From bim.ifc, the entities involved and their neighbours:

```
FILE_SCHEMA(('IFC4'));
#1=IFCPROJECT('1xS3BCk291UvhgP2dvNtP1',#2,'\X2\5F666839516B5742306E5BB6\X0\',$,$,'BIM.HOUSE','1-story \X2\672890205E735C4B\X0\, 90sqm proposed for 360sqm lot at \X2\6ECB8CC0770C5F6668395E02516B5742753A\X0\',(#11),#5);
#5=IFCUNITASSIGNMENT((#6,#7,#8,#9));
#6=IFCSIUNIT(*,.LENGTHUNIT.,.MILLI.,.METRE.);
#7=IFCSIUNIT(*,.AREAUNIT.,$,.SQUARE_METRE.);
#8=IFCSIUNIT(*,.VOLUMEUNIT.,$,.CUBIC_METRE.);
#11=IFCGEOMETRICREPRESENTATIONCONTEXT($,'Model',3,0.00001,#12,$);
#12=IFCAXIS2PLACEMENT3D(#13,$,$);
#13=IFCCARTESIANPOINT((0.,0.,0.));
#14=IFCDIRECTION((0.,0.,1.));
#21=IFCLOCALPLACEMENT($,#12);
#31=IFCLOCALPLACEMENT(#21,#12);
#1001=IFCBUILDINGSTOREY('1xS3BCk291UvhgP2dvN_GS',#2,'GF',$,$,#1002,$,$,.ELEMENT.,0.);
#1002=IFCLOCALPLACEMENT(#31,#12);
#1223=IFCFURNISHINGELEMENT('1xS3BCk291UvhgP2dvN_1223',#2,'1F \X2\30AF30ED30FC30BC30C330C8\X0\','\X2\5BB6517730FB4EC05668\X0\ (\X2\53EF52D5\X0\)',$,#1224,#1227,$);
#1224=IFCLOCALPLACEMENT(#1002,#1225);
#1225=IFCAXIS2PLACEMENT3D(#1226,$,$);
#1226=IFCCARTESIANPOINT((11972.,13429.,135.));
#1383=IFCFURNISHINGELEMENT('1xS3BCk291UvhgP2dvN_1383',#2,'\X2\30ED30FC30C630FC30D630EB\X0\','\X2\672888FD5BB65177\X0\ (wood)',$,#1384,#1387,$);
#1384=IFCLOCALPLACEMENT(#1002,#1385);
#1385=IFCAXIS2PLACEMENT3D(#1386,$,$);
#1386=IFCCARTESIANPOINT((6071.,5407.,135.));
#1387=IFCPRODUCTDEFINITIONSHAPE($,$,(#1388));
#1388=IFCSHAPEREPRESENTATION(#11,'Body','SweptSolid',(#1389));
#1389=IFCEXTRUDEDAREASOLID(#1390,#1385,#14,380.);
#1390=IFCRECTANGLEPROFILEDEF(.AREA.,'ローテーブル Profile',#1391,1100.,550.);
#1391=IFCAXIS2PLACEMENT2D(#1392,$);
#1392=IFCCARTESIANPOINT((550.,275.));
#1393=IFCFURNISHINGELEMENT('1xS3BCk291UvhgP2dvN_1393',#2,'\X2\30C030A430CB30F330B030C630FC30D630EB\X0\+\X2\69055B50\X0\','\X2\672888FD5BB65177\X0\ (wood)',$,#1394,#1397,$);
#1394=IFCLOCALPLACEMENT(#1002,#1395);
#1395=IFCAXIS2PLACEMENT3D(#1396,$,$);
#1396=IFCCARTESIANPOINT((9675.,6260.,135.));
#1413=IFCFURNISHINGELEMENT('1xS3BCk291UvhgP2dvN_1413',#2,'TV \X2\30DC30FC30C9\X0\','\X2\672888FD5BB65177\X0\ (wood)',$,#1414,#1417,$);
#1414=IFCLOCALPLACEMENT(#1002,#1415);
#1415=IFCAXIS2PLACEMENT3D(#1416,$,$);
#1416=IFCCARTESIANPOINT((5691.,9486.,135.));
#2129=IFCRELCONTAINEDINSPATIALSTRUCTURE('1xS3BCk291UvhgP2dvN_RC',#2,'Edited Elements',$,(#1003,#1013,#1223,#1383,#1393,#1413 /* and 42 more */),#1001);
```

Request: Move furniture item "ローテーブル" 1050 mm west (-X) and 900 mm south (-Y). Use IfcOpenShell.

```python
import ifcopenshell
import ifcopenshell.api.geometry
import ifcopenshell.util.placement

model = ifcopenshell.open("bim.ifc")

item = model.by_id(1383)
matrix = ifcopenshell.util.placement.get_local_placement(item.ObjectPlacement)
matrix[0, 3] -= 1050.0
matrix[1, 3] -= 900.0
ifcopenshell.api.geometry.edit_object_placement(model, product=item, matrix=matrix, is_si=False)

print(ifcopenshell.util.placement.get_local_placement(item.ObjectPlacement).round(3) + 0.0)

model.write("bim_rev.ifc")
```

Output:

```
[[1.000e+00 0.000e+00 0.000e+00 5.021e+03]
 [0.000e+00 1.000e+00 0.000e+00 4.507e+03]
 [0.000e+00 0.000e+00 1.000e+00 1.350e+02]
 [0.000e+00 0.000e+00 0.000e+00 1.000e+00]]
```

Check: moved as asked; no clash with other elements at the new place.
